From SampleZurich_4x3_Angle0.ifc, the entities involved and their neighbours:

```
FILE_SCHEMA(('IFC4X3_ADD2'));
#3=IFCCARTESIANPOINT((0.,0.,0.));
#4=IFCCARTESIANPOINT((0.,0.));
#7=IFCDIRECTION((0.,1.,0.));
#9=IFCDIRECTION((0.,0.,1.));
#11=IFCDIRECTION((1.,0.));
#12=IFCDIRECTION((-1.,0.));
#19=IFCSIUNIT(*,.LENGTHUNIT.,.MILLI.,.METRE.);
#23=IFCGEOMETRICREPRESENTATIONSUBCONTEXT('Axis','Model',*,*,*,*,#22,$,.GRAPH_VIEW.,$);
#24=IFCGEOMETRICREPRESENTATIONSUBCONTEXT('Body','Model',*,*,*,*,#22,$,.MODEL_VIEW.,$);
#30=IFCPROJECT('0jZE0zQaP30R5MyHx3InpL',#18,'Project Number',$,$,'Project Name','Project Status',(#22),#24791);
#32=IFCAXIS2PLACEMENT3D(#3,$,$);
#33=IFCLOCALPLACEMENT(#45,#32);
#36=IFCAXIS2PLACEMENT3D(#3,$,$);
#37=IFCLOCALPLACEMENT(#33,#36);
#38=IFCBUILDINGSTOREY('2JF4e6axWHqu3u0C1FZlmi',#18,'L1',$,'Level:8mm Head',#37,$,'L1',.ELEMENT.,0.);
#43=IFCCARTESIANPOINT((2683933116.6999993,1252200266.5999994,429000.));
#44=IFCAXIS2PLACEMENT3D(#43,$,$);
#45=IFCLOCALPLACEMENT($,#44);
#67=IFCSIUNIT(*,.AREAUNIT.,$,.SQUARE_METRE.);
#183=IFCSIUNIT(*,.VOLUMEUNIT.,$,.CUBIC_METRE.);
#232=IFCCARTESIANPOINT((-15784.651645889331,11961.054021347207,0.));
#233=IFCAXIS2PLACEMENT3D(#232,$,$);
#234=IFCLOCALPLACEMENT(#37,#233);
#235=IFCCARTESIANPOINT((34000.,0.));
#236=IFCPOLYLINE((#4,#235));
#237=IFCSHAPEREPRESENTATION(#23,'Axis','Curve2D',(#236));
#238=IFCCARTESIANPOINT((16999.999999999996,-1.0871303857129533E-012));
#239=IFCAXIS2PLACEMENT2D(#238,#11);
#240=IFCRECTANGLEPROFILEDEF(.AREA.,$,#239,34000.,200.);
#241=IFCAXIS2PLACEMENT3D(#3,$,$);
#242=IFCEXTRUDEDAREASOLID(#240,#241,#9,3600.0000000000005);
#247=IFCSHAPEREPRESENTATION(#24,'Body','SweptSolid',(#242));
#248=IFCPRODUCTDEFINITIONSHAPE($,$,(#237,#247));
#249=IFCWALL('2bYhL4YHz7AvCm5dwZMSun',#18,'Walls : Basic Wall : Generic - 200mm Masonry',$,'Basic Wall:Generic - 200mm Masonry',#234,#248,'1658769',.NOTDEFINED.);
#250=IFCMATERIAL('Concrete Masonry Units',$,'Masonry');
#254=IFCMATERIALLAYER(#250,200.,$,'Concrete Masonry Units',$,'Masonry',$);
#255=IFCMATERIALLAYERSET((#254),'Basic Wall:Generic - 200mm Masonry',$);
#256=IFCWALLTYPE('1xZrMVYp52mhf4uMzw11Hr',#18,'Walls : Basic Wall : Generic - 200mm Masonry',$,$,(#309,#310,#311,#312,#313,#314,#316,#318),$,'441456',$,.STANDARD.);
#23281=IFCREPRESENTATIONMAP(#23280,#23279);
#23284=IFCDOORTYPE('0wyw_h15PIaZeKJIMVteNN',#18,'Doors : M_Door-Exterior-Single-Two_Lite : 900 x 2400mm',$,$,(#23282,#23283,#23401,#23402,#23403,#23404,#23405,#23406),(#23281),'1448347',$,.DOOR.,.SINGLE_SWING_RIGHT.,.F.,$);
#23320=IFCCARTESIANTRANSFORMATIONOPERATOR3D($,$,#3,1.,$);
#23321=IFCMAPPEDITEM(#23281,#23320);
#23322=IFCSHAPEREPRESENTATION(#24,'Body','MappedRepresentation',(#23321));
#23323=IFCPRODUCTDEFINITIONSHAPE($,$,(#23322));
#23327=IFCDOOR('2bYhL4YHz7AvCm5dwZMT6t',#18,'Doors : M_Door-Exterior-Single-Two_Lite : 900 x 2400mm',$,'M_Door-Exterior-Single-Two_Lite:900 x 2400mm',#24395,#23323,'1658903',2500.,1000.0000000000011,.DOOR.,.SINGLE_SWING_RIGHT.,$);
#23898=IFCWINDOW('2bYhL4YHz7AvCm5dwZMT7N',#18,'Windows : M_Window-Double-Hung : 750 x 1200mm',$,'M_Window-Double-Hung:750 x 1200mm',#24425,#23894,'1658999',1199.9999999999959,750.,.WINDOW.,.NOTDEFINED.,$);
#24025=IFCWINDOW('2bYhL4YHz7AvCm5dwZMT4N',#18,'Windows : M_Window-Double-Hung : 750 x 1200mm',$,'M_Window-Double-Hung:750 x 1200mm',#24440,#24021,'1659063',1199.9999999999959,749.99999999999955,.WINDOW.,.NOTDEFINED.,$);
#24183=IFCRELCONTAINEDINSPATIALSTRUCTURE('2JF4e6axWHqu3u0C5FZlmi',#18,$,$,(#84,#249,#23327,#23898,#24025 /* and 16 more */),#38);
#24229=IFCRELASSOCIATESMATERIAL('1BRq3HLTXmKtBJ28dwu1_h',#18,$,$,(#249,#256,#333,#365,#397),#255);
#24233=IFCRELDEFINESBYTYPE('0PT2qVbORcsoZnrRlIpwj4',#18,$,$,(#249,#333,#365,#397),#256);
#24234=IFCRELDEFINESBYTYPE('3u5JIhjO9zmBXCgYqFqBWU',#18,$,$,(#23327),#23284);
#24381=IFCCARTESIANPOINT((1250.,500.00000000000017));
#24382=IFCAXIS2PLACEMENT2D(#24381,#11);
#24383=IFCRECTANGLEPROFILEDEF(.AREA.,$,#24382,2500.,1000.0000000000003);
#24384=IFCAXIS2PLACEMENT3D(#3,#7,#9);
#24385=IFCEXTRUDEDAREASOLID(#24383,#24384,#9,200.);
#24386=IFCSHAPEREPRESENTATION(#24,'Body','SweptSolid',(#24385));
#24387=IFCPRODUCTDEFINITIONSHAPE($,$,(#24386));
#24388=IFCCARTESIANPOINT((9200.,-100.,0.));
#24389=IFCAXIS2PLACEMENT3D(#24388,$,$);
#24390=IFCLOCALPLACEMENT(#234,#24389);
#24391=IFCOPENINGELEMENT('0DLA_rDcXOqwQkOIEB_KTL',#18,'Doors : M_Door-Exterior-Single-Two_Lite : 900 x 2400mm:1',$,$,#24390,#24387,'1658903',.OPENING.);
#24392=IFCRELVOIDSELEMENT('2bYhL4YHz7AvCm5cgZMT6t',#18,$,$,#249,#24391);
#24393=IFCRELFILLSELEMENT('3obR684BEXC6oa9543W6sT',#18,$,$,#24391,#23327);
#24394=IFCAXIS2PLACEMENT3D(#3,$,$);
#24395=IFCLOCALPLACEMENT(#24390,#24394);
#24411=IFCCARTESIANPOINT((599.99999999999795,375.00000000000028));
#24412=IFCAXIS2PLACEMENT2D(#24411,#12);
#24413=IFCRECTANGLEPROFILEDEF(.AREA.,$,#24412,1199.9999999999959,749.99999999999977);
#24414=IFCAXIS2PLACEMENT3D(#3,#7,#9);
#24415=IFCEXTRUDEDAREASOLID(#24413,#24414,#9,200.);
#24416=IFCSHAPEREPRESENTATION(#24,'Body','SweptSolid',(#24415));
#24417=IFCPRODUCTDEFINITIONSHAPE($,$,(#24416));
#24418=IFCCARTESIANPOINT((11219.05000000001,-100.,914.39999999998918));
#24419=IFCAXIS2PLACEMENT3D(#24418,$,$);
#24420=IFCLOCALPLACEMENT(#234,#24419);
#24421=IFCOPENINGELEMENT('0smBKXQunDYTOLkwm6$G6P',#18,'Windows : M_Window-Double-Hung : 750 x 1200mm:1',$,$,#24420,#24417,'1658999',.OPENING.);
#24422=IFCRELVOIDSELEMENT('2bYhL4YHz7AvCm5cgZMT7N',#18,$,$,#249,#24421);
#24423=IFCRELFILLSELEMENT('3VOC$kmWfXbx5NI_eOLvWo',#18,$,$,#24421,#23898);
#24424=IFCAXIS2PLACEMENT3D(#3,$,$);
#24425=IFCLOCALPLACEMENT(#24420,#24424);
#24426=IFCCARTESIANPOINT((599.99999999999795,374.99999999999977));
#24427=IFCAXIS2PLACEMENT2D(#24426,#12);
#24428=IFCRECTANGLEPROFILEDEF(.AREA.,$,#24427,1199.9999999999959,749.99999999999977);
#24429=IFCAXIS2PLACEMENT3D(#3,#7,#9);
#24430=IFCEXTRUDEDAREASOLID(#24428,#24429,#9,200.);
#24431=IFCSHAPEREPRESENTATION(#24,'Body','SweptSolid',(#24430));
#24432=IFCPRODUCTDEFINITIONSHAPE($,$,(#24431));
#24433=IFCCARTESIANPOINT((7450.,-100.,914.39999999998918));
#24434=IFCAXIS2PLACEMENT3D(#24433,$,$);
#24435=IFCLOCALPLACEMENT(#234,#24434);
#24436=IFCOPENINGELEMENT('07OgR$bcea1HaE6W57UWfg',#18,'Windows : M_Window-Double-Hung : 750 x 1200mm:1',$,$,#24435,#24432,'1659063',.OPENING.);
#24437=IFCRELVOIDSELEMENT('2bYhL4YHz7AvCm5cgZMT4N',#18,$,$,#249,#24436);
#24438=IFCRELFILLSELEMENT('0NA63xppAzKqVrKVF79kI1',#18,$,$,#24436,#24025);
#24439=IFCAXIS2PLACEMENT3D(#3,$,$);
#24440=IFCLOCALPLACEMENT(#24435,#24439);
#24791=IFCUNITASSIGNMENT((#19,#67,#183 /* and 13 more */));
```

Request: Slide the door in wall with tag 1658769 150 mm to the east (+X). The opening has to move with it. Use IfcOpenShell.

```python
import ifcopenshell
import ifcopenshell.api.geometry
import ifcopenshell.util.placement
import ifcopenshell.util.unit

model = ifcopenshell.open("SampleZurich_4x3_Angle0.ifc")
unit_scale = ifcopenshell.util.unit.calculate_unit_scale(model)

door = model.by_guid("2bYhL4YHz7AvCm5dwZMT6t")
opening = door.FillsVoids[0].RelatingOpeningElement
wall = opening.VoidsElements[0].RelatingBuildingElement

wall_matrix = ifcopenshell.util.placement.get_local_placement(wall.ObjectPlacement)
shift = wall_matrix[:3, 0] * 0.15 / unit_scale
before = ifcopenshell.util.placement.get_local_placement(door.ObjectPlacement)[:3, 3].copy()

# The door is placed relative to its opening, so it follows when the opening moves.
matrix = ifcopenshell.util.placement.get_local_placement(opening.ObjectPlacement)
matrix[:3, 3] += shift
ifcopenshell.api.geometry.edit_object_placement(
    model, product=opening, matrix=matrix, is_si=False, should_transform_children=True
)

after = ifcopenshell.util.placement.get_local_placement(door.ObjectPlacement)[:3, 3]
print("door moved by", (after - before).round(3) + 0.0)

model.write("SampleZurich_4x3_Angle0_updated.ifc")
```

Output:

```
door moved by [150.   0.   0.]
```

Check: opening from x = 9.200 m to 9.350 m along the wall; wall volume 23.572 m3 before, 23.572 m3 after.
